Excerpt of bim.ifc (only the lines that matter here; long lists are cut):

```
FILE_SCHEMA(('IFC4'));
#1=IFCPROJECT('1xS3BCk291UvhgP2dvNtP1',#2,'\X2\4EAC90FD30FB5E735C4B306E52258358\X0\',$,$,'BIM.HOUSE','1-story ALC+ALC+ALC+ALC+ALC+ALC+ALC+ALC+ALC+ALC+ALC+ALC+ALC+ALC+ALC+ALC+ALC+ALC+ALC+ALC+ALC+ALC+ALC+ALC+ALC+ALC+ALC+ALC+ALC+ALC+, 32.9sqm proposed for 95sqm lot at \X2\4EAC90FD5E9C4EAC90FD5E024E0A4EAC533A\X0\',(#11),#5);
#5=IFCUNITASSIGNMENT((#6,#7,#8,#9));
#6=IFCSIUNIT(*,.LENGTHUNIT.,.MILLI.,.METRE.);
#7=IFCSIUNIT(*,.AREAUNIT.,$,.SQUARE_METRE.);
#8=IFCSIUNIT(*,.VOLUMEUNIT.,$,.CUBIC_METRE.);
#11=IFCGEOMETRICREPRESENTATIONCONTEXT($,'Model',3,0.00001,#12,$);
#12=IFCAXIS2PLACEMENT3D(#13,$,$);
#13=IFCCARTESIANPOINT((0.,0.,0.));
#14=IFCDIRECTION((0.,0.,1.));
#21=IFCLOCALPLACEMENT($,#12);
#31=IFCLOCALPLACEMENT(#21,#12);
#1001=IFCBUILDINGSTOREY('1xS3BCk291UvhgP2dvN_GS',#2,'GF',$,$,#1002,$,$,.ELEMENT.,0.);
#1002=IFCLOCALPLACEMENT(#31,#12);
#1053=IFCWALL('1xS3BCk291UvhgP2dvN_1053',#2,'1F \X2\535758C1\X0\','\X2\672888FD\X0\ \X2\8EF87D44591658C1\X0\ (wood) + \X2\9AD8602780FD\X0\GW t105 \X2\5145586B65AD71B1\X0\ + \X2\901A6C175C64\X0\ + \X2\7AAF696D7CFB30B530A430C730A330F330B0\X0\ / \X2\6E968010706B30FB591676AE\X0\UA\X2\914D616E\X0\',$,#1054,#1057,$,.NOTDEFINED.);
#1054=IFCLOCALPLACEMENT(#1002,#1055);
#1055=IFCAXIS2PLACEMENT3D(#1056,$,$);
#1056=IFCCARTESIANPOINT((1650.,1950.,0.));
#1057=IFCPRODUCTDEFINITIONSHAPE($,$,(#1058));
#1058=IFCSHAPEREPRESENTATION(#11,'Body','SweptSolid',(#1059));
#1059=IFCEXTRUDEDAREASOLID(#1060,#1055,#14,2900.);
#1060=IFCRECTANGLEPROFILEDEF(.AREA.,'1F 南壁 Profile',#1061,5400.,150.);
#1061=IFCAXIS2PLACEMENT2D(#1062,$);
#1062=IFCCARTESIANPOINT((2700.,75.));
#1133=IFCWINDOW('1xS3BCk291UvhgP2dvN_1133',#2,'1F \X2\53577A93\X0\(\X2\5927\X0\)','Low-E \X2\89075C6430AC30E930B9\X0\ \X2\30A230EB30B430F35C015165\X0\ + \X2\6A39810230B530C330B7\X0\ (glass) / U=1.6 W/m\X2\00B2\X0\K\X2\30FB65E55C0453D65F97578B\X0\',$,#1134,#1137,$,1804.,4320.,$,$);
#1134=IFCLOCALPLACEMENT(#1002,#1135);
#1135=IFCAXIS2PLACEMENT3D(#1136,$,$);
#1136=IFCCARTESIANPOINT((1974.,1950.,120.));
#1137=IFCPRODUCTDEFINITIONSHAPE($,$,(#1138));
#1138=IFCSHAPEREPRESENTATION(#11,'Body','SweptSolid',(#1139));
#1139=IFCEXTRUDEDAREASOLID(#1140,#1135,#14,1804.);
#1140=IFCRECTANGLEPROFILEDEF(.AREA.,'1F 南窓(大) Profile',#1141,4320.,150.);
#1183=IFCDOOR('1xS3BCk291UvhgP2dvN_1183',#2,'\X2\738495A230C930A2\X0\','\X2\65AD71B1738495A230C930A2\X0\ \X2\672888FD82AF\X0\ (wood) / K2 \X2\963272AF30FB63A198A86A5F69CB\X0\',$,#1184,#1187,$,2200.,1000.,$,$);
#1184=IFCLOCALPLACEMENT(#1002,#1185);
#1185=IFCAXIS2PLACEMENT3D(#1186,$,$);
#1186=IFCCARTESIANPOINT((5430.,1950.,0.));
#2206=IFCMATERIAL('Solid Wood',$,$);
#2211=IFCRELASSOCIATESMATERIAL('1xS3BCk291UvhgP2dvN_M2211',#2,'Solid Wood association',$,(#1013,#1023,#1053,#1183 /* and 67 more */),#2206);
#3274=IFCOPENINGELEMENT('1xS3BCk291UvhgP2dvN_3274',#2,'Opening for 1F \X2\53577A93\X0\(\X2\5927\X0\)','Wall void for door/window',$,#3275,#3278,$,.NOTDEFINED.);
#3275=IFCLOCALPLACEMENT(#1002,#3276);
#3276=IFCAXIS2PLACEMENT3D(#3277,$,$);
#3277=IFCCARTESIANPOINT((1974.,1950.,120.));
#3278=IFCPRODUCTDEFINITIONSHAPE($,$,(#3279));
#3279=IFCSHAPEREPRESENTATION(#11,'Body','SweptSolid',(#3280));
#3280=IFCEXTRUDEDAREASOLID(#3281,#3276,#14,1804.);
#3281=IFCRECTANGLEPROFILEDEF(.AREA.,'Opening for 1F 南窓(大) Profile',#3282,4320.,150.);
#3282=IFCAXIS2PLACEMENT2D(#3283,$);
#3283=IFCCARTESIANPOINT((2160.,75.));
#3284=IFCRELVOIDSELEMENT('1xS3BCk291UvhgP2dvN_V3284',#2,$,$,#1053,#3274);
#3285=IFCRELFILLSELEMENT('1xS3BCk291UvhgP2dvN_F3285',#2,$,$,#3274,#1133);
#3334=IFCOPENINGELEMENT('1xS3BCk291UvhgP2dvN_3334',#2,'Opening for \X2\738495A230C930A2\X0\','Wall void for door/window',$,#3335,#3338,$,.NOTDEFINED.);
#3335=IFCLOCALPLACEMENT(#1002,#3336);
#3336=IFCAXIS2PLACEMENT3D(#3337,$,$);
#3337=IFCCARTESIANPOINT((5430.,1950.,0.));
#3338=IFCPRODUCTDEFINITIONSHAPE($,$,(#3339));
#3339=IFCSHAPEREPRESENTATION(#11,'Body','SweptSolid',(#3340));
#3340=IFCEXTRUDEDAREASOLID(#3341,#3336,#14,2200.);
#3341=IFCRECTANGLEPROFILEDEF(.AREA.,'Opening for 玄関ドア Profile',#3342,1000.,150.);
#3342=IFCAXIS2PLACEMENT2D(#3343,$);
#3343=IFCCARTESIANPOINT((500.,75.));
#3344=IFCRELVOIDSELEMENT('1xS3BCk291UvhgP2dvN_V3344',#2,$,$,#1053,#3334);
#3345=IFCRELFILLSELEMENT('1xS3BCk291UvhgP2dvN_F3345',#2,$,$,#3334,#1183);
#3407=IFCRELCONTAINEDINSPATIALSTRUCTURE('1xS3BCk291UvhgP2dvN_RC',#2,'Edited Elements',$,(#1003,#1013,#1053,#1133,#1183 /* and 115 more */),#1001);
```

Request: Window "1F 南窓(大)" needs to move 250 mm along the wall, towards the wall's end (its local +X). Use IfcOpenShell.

```python
import ifcopenshell
import ifcopenshell.api.geometry
import ifcopenshell.util.placement
import ifcopenshell.util.unit

model = ifcopenshell.open("bim.ifc")
unit_scale = ifcopenshell.util.unit.calculate_unit_scale(model)

window = model.by_guid("1xS3BCk291UvhgP2dvN_1133")
opening = window.FillsVoids[0].RelatingOpeningElement
wall = opening.VoidsElements[0].RelatingBuildingElement

wall_matrix = ifcopenshell.util.placement.get_local_placement(wall.ObjectPlacement)
shift = wall_matrix[:3, 0] * 0.25 / unit_scale
before = ifcopenshell.util.placement.get_local_placement(window.ObjectPlacement)[:3, 3].copy()

# The window is not placed relative to its opening, so move both.
for product in (opening, window):
    matrix = ifcopenshell.util.placement.get_local_placement(product.ObjectPlacement)
    matrix[:3, 3] += shift
    ifcopenshell.api.geometry.edit_object_placement(model, product=product, matrix=matrix, is_si=False)

after = ifcopenshell.util.placement.get_local_placement(window.ObjectPlacement)[:3, 3]
print("window moved by", (after - before).round(3) + 0.0)

model.write("bim_edited.ifc")
```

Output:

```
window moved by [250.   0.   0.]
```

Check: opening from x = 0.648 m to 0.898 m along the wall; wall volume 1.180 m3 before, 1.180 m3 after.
